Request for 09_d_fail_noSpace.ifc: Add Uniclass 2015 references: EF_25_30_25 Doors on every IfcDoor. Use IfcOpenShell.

First a look at what the model holds.

```python
import ifcopenshell

model = ifcopenshell.open("09_d_fail_noSpace.ifc")
print(model.schema)
print("classifications:", [c.Name for c in model.by_type("IfcClassification")])
for ifc_class in ("IfcDoor", "IfcRoof", "IfcStair", "IfcWall", "IfcWindow"):
    print(ifc_class, len(model.by_type(ifc_class)))
```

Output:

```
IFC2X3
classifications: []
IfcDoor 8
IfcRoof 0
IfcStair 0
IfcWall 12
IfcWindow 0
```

```python
import ifcopenshell
import ifcopenshell.api.classification

model = ifcopenshell.open("09_d_fail_noSpace.ifc")

# IFC2X3 requires Source and Edition and has no link from the project to the system.
system = model.create_entity("IfcClassification", Source="NBS", Edition="2015", Name="Uniclass 2015")

codes = {
    "IfcDoor": ("EF_25_30_25", "Doors"),
}
for ifc_class, (code, name) in codes.items():
    products = model.by_type(ifc_class)
    ifcopenshell.api.classification.add_reference(
        model, products=products, classification=system, identification=code, name=name
    )
    print(code, len(products))

model.write("09_d_fail_noSpace-out.ifc")
```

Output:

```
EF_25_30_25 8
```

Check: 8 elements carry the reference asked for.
